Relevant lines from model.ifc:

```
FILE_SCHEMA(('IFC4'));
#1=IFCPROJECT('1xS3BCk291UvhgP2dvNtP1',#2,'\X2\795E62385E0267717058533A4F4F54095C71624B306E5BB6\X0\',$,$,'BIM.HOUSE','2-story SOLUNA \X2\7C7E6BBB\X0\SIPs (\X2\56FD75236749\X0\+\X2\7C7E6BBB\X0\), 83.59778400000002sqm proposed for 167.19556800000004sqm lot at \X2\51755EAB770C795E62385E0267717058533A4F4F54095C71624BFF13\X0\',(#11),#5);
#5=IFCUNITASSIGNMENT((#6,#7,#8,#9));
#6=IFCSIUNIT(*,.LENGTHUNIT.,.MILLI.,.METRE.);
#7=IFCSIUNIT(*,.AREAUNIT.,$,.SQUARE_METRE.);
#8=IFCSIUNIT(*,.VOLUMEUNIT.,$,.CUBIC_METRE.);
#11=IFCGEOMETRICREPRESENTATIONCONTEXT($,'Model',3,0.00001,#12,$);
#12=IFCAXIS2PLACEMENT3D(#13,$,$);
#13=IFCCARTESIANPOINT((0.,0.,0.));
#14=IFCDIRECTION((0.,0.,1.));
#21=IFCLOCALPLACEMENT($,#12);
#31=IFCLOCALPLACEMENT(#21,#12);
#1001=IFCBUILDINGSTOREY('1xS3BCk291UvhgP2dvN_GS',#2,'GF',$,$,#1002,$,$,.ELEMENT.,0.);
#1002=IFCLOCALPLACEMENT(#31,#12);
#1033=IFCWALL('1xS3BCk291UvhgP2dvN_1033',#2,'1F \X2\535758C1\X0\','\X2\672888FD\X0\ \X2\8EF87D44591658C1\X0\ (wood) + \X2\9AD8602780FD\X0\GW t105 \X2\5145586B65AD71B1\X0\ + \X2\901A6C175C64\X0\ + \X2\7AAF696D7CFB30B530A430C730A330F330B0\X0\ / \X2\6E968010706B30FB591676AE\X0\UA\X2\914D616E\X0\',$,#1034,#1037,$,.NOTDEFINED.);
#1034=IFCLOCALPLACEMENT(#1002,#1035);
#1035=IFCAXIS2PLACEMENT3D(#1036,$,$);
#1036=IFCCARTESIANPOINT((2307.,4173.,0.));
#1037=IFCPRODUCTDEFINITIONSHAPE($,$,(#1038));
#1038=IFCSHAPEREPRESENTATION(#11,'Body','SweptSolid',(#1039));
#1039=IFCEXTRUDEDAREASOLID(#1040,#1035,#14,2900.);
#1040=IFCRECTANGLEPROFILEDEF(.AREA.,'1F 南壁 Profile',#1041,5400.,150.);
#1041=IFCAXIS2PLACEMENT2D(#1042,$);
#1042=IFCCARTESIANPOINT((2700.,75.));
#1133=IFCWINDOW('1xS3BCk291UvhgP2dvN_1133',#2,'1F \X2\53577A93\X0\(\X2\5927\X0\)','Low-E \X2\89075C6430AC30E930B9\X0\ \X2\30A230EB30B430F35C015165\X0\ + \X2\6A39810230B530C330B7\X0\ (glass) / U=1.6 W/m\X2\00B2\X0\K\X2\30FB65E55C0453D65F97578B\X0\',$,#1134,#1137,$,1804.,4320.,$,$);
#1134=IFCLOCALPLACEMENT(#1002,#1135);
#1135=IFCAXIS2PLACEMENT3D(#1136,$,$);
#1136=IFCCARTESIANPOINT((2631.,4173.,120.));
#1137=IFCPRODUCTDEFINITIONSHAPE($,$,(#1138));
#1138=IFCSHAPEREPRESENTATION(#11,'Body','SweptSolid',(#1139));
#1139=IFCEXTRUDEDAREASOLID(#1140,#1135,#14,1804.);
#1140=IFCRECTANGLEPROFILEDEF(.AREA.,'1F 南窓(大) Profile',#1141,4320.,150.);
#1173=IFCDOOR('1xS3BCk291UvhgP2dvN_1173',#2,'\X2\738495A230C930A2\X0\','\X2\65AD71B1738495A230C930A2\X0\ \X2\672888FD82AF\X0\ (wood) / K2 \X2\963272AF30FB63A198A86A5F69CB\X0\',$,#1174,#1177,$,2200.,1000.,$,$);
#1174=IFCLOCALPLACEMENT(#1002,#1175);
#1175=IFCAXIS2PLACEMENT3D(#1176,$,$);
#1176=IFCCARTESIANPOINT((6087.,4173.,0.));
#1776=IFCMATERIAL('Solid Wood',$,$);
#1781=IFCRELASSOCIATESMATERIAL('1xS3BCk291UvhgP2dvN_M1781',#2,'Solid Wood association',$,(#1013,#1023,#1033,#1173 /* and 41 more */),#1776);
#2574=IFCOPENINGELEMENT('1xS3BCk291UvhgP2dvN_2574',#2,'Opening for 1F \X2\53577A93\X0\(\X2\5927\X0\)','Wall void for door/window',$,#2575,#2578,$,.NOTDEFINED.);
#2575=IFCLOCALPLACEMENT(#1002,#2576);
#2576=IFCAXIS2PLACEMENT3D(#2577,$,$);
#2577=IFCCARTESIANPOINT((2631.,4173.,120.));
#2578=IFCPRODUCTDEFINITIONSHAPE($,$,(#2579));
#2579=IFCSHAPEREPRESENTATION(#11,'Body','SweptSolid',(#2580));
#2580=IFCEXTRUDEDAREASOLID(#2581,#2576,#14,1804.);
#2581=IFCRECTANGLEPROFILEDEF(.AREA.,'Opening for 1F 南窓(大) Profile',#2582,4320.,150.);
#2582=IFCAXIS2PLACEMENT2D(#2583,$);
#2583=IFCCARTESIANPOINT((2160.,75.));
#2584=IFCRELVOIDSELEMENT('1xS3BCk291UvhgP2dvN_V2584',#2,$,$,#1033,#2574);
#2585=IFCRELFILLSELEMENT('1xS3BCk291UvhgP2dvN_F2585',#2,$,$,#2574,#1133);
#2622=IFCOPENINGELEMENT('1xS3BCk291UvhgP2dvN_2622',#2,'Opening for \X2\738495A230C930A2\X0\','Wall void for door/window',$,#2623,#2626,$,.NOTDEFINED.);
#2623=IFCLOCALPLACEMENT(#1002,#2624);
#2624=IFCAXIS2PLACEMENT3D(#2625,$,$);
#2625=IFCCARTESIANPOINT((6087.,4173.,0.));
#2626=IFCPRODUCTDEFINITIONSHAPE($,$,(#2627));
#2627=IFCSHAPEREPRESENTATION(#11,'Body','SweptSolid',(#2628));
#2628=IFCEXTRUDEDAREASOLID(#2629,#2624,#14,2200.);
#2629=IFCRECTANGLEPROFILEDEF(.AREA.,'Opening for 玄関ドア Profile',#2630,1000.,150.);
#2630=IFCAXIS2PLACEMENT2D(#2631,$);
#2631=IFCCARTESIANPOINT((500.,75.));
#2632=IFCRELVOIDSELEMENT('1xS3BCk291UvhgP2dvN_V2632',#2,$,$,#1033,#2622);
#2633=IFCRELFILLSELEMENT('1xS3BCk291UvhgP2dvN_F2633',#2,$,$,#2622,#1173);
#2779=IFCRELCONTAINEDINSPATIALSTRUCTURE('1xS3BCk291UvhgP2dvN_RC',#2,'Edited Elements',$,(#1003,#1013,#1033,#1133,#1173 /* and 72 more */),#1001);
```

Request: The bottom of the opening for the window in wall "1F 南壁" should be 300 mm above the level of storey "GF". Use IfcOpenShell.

```python
import numpy as np
import ifcopenshell
import ifcopenshell.api.geometry
import ifcopenshell.geom
import ifcopenshell.util.element
import ifcopenshell.util.placement
import ifcopenshell.util.shape
import ifcopenshell.util.unit

model = ifcopenshell.open("model.ifc")
unit_scale = ifcopenshell.util.unit.calculate_unit_scale(model)

window = model.by_id(1133)
opening = window.FillsVoids[0].RelatingOpeningElement
storey = ifcopenshell.util.element.get_container(window, ifc_class="IfcBuildingStorey")
level = ifcopenshell.util.placement.get_local_placement(storey.ObjectPlacement)[2, 3]

# The opening's origin need not be at the sill, so measure its lowest point.
shape = ifcopenshell.geom.create_shape(ifcopenshell.geom.settings(), opening)
bottom = ifcopenshell.util.shape.get_shape_bottom_elevation(shape, shape.geometry) / unit_scale
dz = level + 0.3 / unit_scale - bottom

shift = np.array([0.0, 0.0, dz])
# The window is not placed relative to its opening, so move both.
for product in (opening, window):
    matrix = ifcopenshell.util.placement.get_local_placement(product.ObjectPlacement)
    matrix[:3, 3] += shift
    ifcopenshell.api.geometry.edit_object_placement(model, product=product, matrix=matrix, is_si=False)

print(f"moved by {dz * unit_scale:+.3f} m")

model.write("model_updated.ifc")
```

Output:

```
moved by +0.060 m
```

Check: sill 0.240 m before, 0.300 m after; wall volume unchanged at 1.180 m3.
